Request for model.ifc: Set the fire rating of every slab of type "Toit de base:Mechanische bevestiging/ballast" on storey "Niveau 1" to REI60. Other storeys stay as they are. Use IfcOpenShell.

First a look at what the model holds.

```python
import ifcopenshell
import ifcopenshell.util.element

model = ifcopenshell.open("model.ifc")
print(model.schema)
storey = next(s for s in model.by_type("IfcBuildingStorey") if s.Name == "Niveau 1")
slabs = [e for e in ifcopenshell.util.element.get_decomposition(storey) if e.is_a("IfcSlab")]
seen = {}
for e in slabs:
    element_type = ifcopenshell.util.element.get_type(e)
    key = (element_type.Name if element_type != e and element_type else None, ifcopenshell.util.element.get_pset(e, "Pset_SlabCommon", "FireRating"))
    seen[key] = seen.get(key, 0) + 1
for (name, value), count in sorted(seen.items(), key=str):
    print(count, "x", name, "|", value)
```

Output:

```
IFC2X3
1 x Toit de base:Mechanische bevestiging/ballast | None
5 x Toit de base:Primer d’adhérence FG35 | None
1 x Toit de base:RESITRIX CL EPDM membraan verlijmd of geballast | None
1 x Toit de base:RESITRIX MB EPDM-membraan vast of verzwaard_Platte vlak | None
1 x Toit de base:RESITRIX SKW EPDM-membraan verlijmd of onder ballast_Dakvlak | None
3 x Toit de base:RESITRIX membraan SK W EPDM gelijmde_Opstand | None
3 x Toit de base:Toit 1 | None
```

```python
import ifcopenshell
import ifcopenshell.api.pset
import ifcopenshell.util.element

model = ifcopenshell.open("model.ifc")

storey = next(s for s in model.by_type("IfcBuildingStorey") if s.Name == "Niveau 1")
slabs = [e for e in ifcopenshell.util.element.get_decomposition(storey) if e.is_a("IfcSlab")]

count = 0
for e in slabs:
    element_type = ifcopenshell.util.element.get_type(e)
    if element_type in (None, e) or element_type.Name != "Toit de base:Mechanische bevestiging/ballast":
        continue
    # add_pset returns the element's existing set when there is one.
    pset = ifcopenshell.api.pset.add_pset(model, product=e, name="Pset_SlabCommon")
    ifcopenshell.api.pset.edit_pset(model, pset=pset, properties={"FireRating": "REI60"})
    count += 1

print(count, "slabs updated")

model.write("model_rev.ifc")
```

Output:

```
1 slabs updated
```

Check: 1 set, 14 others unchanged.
